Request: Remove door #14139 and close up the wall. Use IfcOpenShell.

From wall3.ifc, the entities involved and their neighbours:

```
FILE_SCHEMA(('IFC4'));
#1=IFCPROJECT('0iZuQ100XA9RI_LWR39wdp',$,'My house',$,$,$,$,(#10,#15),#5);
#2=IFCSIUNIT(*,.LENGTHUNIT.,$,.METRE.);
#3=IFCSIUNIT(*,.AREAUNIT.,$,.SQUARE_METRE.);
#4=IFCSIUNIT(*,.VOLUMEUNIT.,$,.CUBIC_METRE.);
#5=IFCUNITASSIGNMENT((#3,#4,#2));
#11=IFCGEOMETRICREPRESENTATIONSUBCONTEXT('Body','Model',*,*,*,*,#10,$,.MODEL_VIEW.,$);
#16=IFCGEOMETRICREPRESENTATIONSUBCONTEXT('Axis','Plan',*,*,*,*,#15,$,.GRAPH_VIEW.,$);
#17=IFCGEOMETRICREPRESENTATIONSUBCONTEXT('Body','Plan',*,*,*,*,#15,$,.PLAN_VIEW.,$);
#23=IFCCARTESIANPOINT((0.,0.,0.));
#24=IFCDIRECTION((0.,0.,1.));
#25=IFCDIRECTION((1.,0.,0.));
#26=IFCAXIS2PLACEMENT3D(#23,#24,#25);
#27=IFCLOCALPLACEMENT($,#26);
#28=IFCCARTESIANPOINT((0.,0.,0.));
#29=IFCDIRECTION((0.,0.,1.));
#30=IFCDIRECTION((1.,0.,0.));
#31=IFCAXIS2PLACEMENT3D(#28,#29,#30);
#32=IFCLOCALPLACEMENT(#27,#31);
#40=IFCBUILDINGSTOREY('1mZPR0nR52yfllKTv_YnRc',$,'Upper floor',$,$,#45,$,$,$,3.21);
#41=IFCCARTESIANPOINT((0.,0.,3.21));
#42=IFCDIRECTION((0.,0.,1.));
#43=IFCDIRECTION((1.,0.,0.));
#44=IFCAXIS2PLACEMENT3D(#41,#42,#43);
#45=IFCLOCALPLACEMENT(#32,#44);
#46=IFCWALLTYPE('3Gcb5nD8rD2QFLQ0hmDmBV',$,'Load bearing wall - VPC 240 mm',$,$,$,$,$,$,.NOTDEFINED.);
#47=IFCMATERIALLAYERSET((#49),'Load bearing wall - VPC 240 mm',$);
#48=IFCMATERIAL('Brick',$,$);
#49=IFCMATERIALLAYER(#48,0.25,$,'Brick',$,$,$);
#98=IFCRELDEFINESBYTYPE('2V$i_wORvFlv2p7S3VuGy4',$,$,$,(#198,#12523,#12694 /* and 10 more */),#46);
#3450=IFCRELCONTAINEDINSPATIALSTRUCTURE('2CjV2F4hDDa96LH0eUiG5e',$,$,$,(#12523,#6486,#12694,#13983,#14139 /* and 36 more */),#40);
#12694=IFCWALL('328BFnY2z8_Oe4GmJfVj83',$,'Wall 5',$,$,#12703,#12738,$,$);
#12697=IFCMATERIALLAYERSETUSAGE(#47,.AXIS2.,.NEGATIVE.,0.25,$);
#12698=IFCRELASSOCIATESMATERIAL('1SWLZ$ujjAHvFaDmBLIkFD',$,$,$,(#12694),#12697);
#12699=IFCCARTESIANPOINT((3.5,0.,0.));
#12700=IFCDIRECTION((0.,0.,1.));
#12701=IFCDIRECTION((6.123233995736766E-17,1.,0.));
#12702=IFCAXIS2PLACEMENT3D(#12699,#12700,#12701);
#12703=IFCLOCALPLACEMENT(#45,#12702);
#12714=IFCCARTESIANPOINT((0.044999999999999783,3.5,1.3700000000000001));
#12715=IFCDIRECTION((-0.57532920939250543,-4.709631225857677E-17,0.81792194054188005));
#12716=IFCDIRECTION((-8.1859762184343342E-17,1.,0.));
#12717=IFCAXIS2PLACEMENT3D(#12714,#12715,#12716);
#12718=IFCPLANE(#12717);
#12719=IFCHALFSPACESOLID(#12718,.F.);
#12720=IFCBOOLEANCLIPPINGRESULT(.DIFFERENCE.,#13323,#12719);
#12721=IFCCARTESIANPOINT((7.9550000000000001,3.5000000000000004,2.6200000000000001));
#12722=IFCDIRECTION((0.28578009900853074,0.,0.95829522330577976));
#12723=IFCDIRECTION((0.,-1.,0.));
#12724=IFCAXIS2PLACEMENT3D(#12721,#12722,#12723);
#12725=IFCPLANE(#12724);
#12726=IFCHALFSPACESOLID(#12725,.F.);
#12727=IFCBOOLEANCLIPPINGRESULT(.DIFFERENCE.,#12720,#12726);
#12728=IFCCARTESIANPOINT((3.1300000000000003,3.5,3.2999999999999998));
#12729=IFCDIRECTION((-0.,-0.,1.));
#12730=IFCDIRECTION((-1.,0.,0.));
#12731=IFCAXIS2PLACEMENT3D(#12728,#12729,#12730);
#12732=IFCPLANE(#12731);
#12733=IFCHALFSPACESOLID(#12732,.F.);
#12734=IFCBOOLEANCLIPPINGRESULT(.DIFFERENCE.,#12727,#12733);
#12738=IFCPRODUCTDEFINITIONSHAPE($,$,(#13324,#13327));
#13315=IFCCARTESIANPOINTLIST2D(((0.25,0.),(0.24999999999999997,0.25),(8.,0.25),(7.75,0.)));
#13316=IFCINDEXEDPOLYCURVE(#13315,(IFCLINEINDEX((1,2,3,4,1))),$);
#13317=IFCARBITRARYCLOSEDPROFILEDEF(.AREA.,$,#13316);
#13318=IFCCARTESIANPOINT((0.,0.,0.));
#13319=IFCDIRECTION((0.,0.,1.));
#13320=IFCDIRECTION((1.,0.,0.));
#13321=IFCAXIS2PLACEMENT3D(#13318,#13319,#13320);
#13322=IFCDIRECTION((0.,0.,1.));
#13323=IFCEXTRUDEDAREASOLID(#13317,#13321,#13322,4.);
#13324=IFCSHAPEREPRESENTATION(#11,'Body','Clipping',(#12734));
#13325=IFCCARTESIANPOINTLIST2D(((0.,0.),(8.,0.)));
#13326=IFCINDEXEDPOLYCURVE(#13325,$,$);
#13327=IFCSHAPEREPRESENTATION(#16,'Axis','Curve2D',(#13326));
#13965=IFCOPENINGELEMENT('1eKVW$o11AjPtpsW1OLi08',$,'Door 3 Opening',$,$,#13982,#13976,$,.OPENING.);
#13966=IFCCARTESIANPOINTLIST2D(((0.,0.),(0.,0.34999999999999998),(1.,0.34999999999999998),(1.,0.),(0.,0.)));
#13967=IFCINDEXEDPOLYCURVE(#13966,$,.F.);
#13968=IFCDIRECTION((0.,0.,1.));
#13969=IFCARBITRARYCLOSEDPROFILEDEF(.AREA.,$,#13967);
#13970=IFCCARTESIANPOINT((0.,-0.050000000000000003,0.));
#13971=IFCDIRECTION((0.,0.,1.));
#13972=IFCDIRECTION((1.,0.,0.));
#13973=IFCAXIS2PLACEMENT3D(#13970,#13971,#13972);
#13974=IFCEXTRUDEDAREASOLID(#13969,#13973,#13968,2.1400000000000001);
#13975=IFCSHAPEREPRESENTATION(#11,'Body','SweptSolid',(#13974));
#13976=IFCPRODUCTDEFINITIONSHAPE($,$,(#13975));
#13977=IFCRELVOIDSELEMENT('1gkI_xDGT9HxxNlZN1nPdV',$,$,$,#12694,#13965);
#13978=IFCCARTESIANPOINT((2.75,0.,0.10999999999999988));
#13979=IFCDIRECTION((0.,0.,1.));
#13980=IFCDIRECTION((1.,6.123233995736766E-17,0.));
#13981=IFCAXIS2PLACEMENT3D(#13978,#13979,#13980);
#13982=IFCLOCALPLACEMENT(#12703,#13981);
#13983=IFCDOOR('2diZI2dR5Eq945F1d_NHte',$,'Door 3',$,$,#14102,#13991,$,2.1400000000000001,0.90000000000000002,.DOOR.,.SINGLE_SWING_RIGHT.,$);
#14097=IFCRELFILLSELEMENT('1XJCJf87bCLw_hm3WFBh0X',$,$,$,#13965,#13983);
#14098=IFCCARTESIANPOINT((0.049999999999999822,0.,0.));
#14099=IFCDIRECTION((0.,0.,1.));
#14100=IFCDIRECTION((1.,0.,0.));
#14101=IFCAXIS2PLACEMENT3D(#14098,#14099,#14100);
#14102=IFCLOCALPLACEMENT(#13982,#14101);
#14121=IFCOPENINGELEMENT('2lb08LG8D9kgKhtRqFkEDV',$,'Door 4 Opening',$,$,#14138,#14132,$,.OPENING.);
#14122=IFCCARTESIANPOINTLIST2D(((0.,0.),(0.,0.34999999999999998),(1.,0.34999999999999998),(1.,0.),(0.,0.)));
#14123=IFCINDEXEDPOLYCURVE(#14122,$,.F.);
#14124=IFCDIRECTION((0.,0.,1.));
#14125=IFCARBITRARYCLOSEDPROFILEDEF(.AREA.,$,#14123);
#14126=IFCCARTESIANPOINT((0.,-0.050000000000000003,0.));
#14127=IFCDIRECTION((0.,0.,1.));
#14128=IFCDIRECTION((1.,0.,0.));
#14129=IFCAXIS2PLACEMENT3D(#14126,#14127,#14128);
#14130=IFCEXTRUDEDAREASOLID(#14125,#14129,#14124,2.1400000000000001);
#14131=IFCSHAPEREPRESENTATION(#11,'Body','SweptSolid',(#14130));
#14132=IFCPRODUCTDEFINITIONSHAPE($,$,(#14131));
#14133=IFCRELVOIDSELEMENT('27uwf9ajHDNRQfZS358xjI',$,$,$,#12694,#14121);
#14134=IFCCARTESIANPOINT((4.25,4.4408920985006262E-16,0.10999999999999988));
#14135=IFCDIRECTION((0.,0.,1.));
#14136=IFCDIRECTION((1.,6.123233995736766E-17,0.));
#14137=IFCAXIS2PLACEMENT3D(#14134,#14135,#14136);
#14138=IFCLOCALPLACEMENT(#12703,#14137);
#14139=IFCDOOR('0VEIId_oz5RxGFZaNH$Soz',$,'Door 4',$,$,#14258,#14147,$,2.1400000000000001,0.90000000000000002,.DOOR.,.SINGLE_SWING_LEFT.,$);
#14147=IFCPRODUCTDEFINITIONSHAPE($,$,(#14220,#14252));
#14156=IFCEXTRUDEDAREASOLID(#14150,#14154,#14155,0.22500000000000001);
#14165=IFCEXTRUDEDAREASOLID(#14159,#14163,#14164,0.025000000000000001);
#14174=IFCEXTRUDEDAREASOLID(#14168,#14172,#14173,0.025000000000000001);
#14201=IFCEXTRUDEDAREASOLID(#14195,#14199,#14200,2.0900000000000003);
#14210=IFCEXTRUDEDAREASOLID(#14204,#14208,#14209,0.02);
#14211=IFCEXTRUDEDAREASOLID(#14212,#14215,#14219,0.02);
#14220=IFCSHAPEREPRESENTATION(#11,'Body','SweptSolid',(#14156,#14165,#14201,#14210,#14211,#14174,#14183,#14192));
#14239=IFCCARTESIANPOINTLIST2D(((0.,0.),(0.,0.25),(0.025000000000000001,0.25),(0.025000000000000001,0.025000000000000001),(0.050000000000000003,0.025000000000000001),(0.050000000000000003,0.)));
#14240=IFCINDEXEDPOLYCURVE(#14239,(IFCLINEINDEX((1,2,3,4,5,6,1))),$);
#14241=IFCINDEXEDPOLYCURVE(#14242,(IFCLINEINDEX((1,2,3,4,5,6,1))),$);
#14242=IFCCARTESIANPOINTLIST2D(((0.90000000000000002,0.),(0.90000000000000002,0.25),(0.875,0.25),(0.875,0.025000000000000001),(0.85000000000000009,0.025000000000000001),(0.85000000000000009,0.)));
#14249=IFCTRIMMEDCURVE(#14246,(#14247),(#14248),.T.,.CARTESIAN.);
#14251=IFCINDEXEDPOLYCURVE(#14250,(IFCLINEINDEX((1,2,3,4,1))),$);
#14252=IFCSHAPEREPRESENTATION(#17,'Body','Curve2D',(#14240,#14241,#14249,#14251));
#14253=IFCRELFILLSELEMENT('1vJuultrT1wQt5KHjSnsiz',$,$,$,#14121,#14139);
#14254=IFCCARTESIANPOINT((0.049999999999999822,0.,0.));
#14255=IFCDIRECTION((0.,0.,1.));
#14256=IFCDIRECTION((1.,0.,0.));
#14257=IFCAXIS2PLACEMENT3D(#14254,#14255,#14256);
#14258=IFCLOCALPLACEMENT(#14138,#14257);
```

```python
import ifcopenshell
import ifcopenshell.api.feature
import ifcopenshell.api.root
import ifcopenshell.geom
import ifcopenshell.util.shape

model = ifcopenshell.open("wall3.ifc")
settings = ifcopenshell.geom.settings()


def volume(element):
    """Net volume in cubic metres, openings subtracted."""
    shape = ifcopenshell.geom.create_shape(settings, element)
    return ifcopenshell.util.shape.get_volume(shape.geometry)


door = model.by_guid("0VEIId_oz5RxGFZaNH$Soz")
opening = door.FillsVoids[0].RelatingOpeningElement
wall = opening.VoidsElements[0].RelatingBuildingElement
before = volume(wall)

ifcopenshell.api.root.remove_product(model, product=door)
ifcopenshell.api.feature.remove_feature(model, feature=opening)

after = volume(wall)

print(f"wall volume {before:.3f} -> {after:.3f} m3")

model.write("wall3_rev.ifc")
```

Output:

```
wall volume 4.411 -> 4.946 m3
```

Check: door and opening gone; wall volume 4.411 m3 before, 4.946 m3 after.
